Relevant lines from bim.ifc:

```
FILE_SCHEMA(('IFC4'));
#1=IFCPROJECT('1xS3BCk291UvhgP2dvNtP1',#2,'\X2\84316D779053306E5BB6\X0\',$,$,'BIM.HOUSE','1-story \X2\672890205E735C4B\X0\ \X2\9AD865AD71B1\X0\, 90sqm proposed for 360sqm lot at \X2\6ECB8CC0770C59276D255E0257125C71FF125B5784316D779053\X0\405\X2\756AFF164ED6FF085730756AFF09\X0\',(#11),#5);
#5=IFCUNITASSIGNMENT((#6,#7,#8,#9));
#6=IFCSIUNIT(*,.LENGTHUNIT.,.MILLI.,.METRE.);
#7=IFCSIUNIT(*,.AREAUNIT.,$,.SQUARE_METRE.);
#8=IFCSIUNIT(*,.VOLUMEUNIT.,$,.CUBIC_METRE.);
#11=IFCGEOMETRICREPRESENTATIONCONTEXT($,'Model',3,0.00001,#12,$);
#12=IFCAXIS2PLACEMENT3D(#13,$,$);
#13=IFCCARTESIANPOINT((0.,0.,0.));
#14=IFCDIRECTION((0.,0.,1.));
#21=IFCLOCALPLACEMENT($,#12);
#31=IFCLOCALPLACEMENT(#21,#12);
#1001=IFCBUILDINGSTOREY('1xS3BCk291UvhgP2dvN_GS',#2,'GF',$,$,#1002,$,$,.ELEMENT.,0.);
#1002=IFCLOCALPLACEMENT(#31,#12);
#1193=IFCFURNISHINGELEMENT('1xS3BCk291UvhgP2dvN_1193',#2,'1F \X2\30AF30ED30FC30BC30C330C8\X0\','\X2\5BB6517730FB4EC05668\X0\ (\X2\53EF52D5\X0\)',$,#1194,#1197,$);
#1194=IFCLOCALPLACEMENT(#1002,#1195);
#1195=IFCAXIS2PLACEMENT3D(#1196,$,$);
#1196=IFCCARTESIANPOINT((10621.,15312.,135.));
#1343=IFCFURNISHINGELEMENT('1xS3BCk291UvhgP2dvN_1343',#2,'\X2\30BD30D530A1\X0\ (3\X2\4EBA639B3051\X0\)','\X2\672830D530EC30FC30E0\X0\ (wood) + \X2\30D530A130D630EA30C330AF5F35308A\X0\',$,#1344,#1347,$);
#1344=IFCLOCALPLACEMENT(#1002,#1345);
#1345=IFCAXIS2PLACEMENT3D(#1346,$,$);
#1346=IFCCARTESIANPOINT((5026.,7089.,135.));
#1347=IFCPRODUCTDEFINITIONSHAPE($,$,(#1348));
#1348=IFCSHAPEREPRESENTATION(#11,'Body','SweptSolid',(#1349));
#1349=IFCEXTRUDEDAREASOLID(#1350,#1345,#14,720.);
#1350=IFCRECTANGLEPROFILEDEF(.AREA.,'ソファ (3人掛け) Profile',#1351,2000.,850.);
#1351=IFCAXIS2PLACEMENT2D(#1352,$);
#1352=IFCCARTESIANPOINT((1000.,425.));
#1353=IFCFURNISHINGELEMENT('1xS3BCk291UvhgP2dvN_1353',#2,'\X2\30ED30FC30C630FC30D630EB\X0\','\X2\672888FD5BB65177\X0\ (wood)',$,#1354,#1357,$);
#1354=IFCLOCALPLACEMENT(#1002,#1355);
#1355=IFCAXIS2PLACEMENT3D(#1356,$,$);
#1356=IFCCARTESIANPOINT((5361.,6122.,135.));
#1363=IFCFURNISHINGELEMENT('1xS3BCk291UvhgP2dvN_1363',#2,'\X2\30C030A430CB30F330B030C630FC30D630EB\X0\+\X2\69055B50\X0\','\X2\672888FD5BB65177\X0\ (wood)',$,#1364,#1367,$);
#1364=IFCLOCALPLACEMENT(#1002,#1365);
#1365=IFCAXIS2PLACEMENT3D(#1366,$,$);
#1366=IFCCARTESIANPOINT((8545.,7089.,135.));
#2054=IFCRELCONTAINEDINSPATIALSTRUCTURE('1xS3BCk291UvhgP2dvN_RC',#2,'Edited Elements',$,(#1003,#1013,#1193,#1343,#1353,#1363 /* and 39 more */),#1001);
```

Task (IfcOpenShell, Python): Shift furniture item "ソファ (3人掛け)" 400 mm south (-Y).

```python
import ifcopenshell
import ifcopenshell.api.geometry
import ifcopenshell.util.placement

model = ifcopenshell.open("bim.ifc")

item = model.by_guid("1xS3BCk291UvhgP2dvN_1343")
matrix = ifcopenshell.util.placement.get_local_placement(item.ObjectPlacement)
matrix[1, 3] -= 400.0
ifcopenshell.api.geometry.edit_object_placement(model, product=item, matrix=matrix, is_si=False)

print(ifcopenshell.util.placement.get_local_placement(item.ObjectPlacement).round(3) + 0.0)

model.write("bim_edited.ifc")
```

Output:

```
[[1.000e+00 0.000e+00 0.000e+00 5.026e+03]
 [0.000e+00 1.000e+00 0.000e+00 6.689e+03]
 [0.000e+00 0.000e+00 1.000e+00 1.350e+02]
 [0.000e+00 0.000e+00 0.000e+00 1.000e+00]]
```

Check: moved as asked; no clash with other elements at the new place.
